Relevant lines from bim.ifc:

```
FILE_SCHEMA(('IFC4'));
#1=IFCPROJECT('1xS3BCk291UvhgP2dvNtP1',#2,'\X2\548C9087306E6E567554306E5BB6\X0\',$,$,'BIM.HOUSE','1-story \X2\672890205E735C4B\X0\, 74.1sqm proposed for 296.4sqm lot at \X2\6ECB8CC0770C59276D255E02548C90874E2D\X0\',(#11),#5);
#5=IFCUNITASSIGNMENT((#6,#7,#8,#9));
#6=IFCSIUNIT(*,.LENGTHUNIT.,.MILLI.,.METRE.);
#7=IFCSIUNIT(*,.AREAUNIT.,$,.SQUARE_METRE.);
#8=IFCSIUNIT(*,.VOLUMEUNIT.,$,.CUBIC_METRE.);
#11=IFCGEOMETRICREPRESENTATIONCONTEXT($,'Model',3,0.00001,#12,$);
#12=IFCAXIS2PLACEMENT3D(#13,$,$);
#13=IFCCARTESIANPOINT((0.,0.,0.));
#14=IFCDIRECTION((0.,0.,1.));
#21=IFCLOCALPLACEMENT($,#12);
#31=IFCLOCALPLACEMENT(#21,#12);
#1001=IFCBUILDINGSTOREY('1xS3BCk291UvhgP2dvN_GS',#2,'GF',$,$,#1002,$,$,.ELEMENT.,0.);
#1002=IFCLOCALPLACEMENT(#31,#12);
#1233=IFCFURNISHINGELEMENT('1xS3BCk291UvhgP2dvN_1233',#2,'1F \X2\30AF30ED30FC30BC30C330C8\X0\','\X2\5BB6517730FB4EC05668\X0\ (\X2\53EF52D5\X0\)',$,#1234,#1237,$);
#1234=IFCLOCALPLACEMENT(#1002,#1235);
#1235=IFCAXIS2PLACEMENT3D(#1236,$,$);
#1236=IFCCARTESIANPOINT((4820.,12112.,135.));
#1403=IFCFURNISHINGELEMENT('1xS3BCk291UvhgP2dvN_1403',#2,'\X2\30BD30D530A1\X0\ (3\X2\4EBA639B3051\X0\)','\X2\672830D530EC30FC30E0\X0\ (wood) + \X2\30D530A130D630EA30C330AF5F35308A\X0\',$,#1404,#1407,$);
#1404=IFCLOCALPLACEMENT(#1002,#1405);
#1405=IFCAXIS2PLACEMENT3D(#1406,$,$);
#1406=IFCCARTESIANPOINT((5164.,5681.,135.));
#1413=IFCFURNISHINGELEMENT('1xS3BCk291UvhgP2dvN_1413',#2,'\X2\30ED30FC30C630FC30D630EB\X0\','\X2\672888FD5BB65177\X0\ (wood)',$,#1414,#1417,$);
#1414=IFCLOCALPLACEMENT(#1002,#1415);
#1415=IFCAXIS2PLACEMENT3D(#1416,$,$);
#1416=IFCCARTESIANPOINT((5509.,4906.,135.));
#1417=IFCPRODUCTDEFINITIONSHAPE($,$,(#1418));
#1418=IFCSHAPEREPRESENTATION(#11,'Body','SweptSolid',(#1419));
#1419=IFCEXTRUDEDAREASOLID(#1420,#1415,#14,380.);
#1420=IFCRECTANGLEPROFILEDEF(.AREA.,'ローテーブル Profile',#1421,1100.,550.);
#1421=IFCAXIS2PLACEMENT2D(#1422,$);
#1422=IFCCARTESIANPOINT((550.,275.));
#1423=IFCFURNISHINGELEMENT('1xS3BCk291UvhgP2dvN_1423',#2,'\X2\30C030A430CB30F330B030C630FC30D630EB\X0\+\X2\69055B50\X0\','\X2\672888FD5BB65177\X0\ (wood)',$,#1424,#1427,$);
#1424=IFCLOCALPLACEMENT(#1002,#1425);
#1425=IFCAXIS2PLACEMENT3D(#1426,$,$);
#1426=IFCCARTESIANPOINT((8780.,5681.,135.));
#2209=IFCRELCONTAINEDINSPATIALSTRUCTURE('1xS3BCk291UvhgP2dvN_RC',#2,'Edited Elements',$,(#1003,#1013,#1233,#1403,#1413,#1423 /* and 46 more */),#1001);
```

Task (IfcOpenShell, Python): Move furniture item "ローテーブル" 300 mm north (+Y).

```python
import ifcopenshell
import ifcopenshell.api.geometry
import ifcopenshell.util.placement
import ifcopenshell.util.unit

model = ifcopenshell.open("bim.ifc")
unit_scale = ifcopenshell.util.unit.calculate_unit_scale(model)

item = model.by_id(1413)
matrix = ifcopenshell.util.placement.get_local_placement(item.ObjectPlacement)
matrix[1, 3] += 0.3 / unit_scale
ifcopenshell.api.geometry.edit_object_placement(model, product=item, matrix=matrix, is_si=False)

print(ifcopenshell.util.placement.get_local_placement(item.ObjectPlacement).round(3) + 0.0)

model.write("bim_updated.ifc")
```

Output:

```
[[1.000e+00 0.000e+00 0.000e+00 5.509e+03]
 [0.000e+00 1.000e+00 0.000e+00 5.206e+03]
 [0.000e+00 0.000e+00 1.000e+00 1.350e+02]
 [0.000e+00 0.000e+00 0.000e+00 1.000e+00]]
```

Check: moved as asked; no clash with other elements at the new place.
